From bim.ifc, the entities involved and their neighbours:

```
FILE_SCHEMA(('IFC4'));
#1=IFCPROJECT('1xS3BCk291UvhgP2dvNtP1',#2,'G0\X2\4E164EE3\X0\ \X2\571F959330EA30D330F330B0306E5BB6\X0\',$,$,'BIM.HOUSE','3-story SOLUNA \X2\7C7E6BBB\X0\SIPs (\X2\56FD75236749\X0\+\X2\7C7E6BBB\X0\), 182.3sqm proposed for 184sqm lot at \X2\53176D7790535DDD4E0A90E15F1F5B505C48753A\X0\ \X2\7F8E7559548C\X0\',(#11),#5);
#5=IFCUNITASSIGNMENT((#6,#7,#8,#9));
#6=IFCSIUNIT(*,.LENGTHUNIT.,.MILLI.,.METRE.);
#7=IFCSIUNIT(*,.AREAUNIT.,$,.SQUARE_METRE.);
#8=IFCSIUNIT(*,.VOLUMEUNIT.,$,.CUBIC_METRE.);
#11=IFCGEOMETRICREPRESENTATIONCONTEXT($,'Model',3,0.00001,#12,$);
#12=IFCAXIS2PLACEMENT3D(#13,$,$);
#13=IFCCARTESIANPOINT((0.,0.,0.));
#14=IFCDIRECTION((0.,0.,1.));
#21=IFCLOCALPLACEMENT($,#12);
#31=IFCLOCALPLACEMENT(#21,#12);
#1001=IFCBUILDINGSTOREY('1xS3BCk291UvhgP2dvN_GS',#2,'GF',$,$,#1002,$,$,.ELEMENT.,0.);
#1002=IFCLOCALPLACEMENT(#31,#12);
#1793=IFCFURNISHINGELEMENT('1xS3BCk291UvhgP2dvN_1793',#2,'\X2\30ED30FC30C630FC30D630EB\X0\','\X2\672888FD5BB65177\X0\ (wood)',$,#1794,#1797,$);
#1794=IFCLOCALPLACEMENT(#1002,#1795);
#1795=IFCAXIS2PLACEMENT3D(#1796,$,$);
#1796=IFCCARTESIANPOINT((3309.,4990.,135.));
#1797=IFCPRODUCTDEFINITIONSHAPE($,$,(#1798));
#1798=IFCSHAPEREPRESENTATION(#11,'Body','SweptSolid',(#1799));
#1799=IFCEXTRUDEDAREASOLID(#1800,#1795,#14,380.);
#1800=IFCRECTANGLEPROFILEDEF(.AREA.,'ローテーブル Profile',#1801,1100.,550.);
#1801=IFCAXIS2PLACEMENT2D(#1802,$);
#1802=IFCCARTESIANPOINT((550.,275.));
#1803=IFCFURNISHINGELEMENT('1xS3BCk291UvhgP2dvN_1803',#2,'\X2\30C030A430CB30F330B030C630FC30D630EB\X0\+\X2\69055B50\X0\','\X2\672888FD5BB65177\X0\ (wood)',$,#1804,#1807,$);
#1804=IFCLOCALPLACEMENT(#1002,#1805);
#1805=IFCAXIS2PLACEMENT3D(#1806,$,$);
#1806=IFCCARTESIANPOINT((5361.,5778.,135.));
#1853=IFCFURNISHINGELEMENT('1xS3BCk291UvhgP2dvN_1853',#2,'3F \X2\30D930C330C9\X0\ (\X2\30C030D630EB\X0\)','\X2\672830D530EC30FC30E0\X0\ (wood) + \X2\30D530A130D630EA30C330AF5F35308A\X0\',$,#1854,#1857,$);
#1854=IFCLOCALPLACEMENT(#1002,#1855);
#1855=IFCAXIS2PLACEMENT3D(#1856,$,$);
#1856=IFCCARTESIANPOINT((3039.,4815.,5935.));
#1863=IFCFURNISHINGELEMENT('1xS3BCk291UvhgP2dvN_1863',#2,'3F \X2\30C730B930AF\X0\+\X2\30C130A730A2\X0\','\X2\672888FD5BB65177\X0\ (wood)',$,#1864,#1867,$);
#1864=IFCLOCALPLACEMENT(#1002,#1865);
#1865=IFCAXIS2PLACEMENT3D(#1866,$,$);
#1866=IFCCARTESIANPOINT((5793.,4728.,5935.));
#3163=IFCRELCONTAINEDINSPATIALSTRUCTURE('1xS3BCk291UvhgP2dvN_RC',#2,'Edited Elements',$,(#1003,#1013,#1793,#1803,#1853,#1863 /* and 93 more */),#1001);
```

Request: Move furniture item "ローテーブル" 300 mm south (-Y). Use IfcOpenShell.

```python
import ifcopenshell
import ifcopenshell.api.geometry
import ifcopenshell.util.placement

model = ifcopenshell.open("bim.ifc")

item = model.by_id(1793)
matrix = ifcopenshell.util.placement.get_local_placement(item.ObjectPlacement)
matrix[1, 3] -= 300.0
ifcopenshell.api.geometry.edit_object_placement(model, product=item, matrix=matrix, is_si=False)

print(ifcopenshell.util.placement.get_local_placement(item.ObjectPlacement).round(3) + 0.0)

model.write("bim_edited.ifc")
```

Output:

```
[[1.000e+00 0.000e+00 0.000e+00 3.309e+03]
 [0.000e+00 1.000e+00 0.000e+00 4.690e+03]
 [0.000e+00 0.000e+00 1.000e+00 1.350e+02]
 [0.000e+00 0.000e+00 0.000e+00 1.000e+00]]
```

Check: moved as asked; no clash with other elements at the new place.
